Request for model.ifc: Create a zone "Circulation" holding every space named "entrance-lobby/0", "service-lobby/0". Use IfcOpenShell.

First a look at what the model holds.

```python
import ifcopenshell

model = ifcopenshell.open("model.ifc")
print(model.schema)
seen = {}
for space in model.by_type("IfcSpace"):
    seen[space.Name] = seen.get(space.Name, 0) + 1
for name, count in sorted(seen.items(), key=str):
    print(count, "x", name)
print("zones:", [z.Name for z in model.by_type("IfcZone")][:20])
```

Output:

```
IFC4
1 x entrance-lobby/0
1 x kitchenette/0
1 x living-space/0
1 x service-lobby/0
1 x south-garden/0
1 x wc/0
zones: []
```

```python
import ifcopenshell
import ifcopenshell.api.group
import ifcopenshell.api.root

model = ifcopenshell.open("model.ifc")

names = {"entrance-lobby/0", "service-lobby/0"}
spaces = [s for s in model.by_type("IfcSpace") if s.Name in names]

zone = ifcopenshell.api.root.create_entity(model, ifc_class="IfcZone", name="Circulation")
ifcopenshell.api.group.assign_group(model, products=spaces, group=zone)
print(len(spaces), "spaces in", zone.Name)

model.write("model_updated.ifc")
```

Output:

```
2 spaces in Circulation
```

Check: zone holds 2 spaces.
